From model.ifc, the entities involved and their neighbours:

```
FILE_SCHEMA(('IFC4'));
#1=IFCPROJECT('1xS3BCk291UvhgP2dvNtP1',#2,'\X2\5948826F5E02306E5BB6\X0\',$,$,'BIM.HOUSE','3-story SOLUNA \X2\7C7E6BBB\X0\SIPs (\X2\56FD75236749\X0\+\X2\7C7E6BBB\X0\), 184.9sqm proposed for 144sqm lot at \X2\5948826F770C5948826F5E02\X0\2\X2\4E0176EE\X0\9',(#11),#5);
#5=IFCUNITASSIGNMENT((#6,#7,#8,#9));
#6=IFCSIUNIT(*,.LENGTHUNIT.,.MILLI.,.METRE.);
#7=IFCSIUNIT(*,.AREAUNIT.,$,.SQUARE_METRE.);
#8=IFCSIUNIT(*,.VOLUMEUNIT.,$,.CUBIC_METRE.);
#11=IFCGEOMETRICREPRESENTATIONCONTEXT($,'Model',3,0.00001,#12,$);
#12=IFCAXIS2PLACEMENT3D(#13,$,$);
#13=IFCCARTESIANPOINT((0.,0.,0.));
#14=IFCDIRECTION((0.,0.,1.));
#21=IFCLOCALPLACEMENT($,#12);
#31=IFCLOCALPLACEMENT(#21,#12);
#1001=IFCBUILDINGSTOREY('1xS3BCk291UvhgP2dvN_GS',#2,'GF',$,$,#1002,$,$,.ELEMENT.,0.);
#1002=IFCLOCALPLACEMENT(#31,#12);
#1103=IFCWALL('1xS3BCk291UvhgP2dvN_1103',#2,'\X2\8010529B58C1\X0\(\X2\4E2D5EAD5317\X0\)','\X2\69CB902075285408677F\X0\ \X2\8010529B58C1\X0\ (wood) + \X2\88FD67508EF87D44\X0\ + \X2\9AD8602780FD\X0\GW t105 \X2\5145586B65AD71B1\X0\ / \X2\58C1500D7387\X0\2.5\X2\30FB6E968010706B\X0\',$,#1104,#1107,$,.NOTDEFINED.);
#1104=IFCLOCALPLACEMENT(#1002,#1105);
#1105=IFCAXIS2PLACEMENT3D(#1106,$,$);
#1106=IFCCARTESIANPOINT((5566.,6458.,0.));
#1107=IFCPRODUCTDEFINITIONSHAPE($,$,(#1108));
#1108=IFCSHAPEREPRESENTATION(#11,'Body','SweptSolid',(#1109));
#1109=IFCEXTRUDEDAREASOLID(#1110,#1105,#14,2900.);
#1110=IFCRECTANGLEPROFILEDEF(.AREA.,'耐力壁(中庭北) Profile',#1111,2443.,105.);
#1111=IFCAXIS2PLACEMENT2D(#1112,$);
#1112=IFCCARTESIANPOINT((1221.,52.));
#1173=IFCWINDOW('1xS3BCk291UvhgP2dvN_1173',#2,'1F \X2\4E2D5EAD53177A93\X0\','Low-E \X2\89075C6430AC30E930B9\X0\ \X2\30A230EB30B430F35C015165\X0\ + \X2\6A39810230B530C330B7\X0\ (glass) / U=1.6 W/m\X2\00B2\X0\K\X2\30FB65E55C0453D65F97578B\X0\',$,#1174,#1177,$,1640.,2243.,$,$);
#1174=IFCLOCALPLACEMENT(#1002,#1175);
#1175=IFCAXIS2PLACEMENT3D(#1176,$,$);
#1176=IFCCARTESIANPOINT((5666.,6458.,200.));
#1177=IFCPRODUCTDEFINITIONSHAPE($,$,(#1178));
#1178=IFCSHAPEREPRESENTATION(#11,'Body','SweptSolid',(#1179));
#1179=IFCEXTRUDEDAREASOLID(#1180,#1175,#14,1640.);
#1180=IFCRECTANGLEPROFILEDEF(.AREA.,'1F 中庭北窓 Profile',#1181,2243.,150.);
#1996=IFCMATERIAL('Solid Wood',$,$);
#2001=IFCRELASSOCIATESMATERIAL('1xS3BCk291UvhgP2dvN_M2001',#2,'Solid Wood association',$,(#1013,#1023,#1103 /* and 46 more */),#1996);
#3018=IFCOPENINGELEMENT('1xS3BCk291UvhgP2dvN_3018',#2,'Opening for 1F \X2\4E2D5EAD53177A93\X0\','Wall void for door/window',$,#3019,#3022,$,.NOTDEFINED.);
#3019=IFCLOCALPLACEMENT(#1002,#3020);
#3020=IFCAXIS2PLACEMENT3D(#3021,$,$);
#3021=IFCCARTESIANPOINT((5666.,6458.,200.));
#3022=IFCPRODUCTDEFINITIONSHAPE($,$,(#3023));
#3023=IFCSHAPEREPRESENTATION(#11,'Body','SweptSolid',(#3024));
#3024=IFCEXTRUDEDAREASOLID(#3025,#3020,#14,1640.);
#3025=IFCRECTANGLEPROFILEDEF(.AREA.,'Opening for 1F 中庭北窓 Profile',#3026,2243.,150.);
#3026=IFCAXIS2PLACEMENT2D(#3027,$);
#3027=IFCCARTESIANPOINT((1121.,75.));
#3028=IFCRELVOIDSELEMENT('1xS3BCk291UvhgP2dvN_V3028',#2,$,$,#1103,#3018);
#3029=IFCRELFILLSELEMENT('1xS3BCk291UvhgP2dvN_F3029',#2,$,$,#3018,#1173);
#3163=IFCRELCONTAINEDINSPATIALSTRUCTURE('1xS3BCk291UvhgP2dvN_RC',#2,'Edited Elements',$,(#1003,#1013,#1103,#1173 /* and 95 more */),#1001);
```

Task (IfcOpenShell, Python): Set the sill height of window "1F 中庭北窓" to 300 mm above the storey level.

```python
import numpy as np
import ifcopenshell
import ifcopenshell.api.geometry
import ifcopenshell.geom
import ifcopenshell.util.element
import ifcopenshell.util.placement
import ifcopenshell.util.shape
import ifcopenshell.util.unit

model = ifcopenshell.open("model.ifc")
unit_scale = ifcopenshell.util.unit.calculate_unit_scale(model)

window = model.by_id(1173)
opening = window.FillsVoids[0].RelatingOpeningElement
storey = ifcopenshell.util.element.get_container(window, ifc_class="IfcBuildingStorey")
level = ifcopenshell.util.placement.get_local_placement(storey.ObjectPlacement)[2, 3]

# The opening's origin need not be at the sill, so measure its lowest point.
shape = ifcopenshell.geom.create_shape(ifcopenshell.geom.settings(), opening)
bottom = ifcopenshell.util.shape.get_shape_bottom_elevation(shape, shape.geometry) / unit_scale
dz = level + 0.3 / unit_scale - bottom

shift = np.array([0.0, 0.0, dz])
# The window is not placed relative to its opening, so move both.
for product in (opening, window):
    matrix = ifcopenshell.util.placement.get_local_placement(product.ObjectPlacement)
    matrix[:3, 3] += shift
    ifcopenshell.api.geometry.edit_object_placement(model, product=product, matrix=matrix, is_si=False)

print(f"moved by {dz * unit_scale:+.3f} m")

model.write("model_rev.ifc")
```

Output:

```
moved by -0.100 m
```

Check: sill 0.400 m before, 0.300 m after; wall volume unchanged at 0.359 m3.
